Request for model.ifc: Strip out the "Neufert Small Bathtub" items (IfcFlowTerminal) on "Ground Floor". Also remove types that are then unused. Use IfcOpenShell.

First a look at what the model holds.

```python
import ifcopenshell
import ifcopenshell.util.element

model = ifcopenshell.open("model.ifc")
print(model.schema)
storey = next(s for s in model.by_type("IfcBuildingStorey") if s.Name == "Ground Floor")
terminals = [e for e in ifcopenshell.util.element.get_decomposition(storey) if e.is_a("IfcFlowTerminal")]
seen = {}
for e in terminals:
    element_type = ifcopenshell.util.element.get_type(e)
    name = element_type.Name if element_type not in (None, e) else None
    seen[name] = seen.get(name, 0) + 1
for name, count in sorted(seen.items(), key=str):
    print(count, "x", name)
```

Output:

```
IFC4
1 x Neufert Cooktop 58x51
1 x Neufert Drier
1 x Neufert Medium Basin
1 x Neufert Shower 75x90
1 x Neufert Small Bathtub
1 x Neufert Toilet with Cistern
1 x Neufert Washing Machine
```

```python
import ifcopenshell
import ifcopenshell.api.root
import ifcopenshell.util.element

model = ifcopenshell.open("model.ifc")

storey = next(s for s in model.by_type("IfcBuildingStorey") if s.Name == "Ground Floor")
terminals = [e for e in ifcopenshell.util.element.get_decomposition(storey) if e.is_a("IfcFlowTerminal")]
targets = [e for e in terminals if (t := ifcopenshell.util.element.get_type(e)) not in (None, e) and t.Name == "Neufert Small Bathtub"]
types = {ifcopenshell.util.element.get_type(e) for e in targets} - {None, *targets}

for e in targets:
    ifcopenshell.api.root.remove_product(model, product=e)
print(len(targets), "removed")

unused = [t for t in types if not ifcopenshell.util.element.get_types(t)]
for t in unused:
    ifcopenshell.api.root.remove_product(model, product=t)
print(len(unused), "unused types removed")

model.write("model_rev.ifc")
```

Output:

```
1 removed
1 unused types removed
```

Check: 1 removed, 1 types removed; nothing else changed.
